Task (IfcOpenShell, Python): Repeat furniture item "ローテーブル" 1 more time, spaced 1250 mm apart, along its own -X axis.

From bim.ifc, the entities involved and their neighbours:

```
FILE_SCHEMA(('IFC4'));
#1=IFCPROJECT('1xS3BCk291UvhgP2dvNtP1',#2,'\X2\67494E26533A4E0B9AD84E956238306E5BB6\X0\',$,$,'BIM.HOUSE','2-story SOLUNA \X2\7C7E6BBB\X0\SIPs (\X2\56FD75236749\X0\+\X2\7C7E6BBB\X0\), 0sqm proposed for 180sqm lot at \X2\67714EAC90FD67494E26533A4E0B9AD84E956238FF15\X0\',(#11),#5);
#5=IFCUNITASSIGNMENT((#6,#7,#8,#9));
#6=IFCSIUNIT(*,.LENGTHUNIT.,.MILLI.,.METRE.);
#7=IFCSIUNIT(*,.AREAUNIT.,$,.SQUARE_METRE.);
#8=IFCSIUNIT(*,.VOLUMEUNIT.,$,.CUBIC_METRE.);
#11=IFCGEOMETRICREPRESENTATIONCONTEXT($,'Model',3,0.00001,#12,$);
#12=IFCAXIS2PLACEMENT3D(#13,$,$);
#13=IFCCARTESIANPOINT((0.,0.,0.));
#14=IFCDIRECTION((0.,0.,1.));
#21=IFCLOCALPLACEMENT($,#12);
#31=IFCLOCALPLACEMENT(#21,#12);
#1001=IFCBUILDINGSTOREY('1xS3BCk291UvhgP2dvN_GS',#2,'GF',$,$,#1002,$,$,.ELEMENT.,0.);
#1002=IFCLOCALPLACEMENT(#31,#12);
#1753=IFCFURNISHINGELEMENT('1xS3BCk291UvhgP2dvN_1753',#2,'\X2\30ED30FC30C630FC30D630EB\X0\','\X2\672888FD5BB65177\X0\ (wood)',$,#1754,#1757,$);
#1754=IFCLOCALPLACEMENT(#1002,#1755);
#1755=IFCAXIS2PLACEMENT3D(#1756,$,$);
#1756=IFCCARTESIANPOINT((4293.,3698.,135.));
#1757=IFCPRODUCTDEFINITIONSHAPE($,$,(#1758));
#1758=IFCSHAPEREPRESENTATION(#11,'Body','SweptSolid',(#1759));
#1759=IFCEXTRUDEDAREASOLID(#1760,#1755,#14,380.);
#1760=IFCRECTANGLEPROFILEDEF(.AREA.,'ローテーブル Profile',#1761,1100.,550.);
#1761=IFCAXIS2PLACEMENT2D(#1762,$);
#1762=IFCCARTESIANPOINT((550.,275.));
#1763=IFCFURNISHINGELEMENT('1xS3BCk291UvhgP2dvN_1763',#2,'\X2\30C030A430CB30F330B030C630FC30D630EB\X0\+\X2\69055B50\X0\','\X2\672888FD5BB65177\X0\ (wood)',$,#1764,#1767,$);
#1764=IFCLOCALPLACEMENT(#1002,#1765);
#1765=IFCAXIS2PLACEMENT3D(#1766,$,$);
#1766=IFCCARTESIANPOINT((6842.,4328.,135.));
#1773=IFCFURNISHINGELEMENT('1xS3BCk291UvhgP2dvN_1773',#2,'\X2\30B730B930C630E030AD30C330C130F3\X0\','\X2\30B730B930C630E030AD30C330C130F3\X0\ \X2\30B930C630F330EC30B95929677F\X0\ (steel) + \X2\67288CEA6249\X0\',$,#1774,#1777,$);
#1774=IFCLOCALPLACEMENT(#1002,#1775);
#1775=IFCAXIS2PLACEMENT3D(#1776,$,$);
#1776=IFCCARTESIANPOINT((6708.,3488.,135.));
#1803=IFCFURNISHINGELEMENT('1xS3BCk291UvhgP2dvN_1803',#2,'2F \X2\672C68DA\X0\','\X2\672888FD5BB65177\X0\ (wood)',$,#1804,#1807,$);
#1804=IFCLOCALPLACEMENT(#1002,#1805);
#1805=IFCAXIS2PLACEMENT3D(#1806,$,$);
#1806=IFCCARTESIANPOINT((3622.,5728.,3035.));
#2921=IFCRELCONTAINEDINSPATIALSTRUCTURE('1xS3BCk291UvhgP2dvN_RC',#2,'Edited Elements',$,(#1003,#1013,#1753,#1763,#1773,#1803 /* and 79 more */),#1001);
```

```python
import ifcopenshell
import ifcopenshell.api.geometry
import ifcopenshell.api.root
import ifcopenshell.util.element
import ifcopenshell.util.placement
import ifcopenshell.util.unit

model = ifcopenshell.open("bim.ifc")
unit_scale = ifcopenshell.util.unit.calculate_unit_scale(model)


def reuse_history(source, copy):
    """copy_class also copies each property set's owner history, people and application; keep the originals."""
    for rel in copy.IsDefinedBy:
        if rel.is_a("IfcRelDefinesByProperties") and (history := rel.RelatingPropertyDefinition.OwnerHistory):
            rel.RelatingPropertyDefinition.OwnerHistory = source.OwnerHistory
            ifcopenshell.util.element.remove_deep2(model, history)


source = model.by_id(1753)
base = ifcopenshell.util.placement.get_local_placement(source.ObjectPlacement)
step = -base[:3, 0] * 1.25 / unit_scale

for i in range(1, 2):
    copy = ifcopenshell.api.root.copy_class(model, product=source)
    copy.Representation = ifcopenshell.util.element.copy_deep(
        model, source.Representation, exclude=["IfcGeometricRepresentationContext", "IfcRepresentationMap"]
    )
    reuse_history(source, copy)
    matrix = base.copy()
    matrix[:3, 3] += i * step
    print("added at", matrix[:3, 3].round(3) + 0.0)
    ifcopenshell.api.geometry.edit_object_placement(model, product=copy, matrix=matrix, is_si=False)

model.write("bim-out.ifc")
```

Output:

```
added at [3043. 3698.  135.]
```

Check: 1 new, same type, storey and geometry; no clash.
